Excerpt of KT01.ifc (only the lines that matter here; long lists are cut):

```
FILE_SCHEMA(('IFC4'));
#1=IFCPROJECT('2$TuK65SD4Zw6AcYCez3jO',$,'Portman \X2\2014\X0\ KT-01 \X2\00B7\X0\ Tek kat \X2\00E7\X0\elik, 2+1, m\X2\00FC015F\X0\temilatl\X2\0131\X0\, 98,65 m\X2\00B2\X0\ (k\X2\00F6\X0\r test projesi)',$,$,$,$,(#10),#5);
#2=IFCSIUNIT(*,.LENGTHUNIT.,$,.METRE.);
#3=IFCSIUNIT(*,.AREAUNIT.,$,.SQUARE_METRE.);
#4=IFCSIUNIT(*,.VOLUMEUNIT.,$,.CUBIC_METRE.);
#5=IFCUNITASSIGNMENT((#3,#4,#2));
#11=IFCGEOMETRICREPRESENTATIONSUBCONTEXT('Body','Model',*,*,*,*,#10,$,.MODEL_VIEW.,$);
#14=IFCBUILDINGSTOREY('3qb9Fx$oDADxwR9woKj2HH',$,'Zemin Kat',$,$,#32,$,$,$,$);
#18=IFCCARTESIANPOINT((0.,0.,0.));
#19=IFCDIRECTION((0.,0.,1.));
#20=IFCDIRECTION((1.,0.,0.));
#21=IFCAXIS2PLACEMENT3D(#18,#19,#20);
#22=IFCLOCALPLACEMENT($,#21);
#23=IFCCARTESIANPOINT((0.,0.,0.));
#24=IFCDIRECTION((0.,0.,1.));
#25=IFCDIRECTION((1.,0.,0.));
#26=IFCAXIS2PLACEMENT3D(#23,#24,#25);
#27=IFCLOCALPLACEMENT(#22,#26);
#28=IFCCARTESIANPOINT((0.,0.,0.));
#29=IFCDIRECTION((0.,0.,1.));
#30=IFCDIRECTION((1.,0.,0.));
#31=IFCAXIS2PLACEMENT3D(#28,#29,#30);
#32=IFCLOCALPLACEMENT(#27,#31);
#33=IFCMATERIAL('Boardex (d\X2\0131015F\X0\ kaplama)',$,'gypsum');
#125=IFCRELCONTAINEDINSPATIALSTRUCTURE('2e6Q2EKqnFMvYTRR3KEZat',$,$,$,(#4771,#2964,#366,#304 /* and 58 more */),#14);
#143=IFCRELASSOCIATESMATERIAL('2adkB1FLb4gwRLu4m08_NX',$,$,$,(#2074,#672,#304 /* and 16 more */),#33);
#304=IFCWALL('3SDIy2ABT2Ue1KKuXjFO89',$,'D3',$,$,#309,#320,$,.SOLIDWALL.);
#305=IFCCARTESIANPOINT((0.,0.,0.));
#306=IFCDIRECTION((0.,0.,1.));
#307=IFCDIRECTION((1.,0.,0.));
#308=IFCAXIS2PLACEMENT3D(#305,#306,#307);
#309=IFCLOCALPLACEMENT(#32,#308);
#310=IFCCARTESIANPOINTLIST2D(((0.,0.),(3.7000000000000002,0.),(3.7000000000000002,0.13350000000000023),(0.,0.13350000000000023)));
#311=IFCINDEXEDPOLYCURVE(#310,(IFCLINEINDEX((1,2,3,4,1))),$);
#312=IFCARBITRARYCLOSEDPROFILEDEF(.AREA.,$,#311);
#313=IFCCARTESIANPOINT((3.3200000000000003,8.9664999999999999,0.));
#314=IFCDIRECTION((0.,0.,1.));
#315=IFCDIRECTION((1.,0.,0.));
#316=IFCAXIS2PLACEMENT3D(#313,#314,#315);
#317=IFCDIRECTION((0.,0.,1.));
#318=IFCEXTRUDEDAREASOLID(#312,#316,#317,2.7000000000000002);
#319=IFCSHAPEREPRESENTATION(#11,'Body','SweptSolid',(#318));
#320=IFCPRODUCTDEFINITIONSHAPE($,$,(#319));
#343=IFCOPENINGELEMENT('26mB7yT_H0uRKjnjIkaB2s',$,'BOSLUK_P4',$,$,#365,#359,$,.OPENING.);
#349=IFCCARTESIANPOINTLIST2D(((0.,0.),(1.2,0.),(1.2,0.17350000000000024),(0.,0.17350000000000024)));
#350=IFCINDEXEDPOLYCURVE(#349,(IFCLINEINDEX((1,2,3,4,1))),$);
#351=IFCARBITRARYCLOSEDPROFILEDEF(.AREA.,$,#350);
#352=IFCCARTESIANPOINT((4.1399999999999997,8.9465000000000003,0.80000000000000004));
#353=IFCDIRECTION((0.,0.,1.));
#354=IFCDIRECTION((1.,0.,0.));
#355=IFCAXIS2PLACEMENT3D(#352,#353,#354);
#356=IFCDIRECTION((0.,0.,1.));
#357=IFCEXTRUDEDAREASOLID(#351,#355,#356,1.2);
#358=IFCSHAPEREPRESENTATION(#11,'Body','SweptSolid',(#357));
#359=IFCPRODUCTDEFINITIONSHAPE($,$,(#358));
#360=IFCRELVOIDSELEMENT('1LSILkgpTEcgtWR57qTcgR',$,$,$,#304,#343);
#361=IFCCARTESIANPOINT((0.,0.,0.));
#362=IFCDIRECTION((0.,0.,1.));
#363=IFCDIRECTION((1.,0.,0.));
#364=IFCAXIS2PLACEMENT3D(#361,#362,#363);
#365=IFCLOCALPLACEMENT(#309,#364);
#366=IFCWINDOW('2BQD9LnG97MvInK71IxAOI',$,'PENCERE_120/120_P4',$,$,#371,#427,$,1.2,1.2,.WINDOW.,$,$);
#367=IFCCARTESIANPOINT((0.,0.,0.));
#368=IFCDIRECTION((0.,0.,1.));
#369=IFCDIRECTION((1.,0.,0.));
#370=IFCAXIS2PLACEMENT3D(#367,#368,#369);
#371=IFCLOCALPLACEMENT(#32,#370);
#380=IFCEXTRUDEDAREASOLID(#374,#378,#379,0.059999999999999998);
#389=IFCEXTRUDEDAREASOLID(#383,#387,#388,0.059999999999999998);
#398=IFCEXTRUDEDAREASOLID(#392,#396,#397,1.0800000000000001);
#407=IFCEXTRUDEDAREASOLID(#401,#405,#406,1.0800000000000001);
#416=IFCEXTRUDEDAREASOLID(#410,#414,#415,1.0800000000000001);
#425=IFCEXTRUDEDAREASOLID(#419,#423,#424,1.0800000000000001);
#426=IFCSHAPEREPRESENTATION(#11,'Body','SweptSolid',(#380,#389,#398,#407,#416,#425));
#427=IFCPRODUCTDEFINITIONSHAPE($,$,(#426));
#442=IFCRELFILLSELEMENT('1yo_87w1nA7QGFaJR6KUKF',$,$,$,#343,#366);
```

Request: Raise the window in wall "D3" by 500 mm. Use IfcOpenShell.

```python
import numpy as np
import ifcopenshell
import ifcopenshell.api.geometry
import ifcopenshell.util.placement
import ifcopenshell.util.unit

model = ifcopenshell.open("KT01.ifc")
unit_scale = ifcopenshell.util.unit.calculate_unit_scale(model)

window = model.by_guid("2BQD9LnG97MvInK71IxAOI")
opening = window.FillsVoids[0].RelatingOpeningElement
dz = 0.5 / unit_scale

shift = np.array([0.0, 0.0, dz])
# The window is not placed relative to its opening, so move both.
for product in (opening, window):
    matrix = ifcopenshell.util.placement.get_local_placement(product.ObjectPlacement)
    matrix[:3, 3] += shift
    ifcopenshell.api.geometry.edit_object_placement(model, product=product, matrix=matrix, is_si=False)

print(f"moved by {dz * unit_scale:+.3f} m")

model.write("KT01_updated.ifc")
```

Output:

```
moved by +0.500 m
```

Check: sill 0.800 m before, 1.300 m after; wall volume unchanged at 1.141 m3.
